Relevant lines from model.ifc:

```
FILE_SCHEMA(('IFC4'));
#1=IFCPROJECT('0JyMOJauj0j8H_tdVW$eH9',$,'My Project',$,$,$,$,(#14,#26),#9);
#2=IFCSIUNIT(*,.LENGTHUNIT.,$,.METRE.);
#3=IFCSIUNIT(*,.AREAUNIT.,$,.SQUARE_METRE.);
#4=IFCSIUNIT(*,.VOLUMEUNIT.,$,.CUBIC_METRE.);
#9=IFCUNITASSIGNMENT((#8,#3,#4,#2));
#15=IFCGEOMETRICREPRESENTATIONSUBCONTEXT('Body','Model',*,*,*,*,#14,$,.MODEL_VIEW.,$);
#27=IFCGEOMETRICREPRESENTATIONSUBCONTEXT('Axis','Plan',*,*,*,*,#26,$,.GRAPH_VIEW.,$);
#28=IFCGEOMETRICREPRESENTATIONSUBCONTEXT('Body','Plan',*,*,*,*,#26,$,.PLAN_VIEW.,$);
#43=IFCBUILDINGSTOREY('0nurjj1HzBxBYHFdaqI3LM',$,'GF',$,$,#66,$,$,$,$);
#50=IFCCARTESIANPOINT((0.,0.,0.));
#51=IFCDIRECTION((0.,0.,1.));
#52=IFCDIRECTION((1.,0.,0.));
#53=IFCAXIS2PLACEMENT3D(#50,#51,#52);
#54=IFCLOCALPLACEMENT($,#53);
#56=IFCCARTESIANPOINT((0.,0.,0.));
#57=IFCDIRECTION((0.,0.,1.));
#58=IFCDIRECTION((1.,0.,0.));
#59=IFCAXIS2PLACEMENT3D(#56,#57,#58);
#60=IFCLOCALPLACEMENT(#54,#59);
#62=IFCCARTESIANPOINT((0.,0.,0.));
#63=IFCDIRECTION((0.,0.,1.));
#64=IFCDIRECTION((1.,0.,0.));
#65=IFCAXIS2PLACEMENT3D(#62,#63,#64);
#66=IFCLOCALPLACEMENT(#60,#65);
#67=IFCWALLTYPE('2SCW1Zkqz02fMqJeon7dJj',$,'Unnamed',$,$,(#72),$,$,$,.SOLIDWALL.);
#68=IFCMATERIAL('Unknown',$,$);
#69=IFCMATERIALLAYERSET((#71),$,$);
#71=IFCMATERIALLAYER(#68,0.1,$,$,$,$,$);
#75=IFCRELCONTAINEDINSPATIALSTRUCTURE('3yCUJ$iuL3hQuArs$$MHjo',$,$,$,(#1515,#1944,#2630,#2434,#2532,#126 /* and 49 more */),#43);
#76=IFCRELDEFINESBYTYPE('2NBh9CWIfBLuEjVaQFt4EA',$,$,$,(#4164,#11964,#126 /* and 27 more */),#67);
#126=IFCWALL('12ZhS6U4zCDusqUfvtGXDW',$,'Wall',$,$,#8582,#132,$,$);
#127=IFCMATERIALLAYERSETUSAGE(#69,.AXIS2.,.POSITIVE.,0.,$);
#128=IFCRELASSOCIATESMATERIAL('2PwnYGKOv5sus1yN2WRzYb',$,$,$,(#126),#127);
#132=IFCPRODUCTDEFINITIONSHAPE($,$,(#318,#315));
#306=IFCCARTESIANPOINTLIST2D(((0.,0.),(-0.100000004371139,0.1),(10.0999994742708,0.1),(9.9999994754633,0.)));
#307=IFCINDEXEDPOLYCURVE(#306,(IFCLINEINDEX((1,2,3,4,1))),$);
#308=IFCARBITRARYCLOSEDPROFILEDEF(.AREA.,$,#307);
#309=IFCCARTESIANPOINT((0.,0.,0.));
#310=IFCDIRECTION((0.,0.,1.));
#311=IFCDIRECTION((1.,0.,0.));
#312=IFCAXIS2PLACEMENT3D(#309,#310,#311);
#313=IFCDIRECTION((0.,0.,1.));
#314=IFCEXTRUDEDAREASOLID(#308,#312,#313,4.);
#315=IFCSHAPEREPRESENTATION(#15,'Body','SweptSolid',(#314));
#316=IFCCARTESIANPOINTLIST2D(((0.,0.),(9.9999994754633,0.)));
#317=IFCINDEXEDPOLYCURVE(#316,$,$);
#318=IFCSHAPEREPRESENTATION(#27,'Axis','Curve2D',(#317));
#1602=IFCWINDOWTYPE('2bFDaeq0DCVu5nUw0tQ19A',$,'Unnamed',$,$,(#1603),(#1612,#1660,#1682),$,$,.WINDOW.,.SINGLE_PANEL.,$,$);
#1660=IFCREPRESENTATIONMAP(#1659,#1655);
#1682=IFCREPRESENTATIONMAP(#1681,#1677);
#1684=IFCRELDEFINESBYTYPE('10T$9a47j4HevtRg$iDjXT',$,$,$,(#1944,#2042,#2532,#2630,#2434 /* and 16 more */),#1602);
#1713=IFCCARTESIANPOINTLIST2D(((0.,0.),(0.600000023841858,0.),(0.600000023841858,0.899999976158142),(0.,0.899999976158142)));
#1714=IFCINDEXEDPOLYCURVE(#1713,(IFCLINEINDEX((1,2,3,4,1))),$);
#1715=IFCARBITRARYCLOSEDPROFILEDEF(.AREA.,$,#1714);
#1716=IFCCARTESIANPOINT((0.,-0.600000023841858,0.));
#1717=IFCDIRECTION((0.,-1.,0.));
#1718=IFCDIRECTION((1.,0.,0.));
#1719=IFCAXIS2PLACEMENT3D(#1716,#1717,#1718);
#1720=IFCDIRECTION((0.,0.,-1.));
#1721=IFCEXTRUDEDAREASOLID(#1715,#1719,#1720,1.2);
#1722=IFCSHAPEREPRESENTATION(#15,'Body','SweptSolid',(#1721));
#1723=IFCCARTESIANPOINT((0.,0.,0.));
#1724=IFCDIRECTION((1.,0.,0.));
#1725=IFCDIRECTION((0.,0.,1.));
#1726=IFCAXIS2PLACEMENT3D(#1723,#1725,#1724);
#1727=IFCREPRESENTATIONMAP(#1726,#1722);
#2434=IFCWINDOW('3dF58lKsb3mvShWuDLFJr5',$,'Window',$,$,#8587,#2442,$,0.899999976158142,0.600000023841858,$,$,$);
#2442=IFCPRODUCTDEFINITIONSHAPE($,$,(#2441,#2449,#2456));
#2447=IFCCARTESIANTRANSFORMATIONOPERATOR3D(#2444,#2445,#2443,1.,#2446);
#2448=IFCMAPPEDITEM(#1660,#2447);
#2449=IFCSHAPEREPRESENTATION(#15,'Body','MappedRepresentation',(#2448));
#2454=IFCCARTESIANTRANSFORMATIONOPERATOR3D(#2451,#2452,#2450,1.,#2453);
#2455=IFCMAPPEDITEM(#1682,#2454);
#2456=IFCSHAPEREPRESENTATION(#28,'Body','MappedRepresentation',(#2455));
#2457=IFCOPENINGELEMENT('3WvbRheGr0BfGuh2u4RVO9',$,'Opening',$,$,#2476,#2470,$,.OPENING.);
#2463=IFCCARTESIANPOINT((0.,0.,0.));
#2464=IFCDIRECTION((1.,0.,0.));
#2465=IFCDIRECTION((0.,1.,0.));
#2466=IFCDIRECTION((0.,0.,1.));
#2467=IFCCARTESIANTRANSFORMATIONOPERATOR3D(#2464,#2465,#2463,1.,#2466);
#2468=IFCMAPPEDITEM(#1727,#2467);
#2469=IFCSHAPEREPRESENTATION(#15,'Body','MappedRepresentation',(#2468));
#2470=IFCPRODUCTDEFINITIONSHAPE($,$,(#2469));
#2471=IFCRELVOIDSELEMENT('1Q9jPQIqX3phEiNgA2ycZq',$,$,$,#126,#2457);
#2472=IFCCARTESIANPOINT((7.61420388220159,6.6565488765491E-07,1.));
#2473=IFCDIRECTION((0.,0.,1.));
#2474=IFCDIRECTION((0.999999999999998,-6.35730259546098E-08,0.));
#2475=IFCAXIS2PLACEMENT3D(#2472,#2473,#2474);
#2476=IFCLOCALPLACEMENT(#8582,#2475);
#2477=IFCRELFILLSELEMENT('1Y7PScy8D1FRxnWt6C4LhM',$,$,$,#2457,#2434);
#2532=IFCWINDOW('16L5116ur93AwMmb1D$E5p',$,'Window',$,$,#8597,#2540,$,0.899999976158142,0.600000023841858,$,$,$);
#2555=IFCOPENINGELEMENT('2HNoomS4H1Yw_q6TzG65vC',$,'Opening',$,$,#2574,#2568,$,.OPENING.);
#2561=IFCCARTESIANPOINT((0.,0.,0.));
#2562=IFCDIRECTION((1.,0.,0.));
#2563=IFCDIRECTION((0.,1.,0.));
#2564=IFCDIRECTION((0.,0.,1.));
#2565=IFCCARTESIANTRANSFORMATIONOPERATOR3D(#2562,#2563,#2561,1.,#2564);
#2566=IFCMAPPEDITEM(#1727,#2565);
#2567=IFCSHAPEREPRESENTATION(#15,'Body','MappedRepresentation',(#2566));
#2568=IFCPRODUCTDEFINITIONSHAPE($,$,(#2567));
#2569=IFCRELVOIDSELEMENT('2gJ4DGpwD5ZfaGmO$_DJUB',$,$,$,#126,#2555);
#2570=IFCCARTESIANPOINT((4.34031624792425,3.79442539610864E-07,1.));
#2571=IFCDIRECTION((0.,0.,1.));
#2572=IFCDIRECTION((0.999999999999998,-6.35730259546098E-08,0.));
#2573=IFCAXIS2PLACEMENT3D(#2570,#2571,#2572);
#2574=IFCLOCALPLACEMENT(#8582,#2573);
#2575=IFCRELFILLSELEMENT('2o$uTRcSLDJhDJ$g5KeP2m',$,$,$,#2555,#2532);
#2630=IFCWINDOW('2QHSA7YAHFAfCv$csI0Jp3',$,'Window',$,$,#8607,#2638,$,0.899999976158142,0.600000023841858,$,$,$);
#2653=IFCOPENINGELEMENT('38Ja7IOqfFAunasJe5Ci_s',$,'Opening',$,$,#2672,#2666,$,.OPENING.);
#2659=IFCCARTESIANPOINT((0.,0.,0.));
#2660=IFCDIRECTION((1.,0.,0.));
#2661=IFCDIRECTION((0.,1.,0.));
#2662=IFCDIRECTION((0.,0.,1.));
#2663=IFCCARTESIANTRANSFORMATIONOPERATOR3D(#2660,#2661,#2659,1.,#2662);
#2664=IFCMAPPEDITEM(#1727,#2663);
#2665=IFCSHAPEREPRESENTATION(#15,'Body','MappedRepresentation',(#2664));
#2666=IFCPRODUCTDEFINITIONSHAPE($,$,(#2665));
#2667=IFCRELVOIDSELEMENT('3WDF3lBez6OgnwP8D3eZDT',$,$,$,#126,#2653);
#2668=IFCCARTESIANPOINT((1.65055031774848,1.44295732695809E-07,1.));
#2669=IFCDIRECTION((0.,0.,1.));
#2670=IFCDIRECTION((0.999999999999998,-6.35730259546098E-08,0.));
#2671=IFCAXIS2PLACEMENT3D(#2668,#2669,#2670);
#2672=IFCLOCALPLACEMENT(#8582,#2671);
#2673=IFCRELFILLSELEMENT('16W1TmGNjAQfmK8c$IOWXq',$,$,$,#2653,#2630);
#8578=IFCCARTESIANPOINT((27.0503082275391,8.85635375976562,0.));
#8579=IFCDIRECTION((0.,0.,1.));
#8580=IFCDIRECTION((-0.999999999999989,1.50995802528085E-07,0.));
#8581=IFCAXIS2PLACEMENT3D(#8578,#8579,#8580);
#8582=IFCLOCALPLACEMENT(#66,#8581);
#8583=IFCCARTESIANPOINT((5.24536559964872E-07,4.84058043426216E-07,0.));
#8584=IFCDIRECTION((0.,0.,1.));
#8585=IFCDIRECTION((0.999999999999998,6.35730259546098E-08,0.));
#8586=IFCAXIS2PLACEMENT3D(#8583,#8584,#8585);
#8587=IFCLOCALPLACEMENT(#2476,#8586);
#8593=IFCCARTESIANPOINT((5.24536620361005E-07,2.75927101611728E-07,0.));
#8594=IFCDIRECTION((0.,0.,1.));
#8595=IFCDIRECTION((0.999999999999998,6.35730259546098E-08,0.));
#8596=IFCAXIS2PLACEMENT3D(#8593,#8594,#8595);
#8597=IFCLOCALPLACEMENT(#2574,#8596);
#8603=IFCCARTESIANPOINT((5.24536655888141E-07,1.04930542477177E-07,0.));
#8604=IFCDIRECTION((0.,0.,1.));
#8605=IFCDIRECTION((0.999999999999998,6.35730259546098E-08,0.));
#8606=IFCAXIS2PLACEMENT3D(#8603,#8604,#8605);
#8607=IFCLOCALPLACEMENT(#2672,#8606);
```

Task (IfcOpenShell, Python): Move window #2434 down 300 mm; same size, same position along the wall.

```python
import numpy as np
import ifcopenshell
import ifcopenshell.api.geometry
import ifcopenshell.util.placement
import ifcopenshell.util.unit

model = ifcopenshell.open("model.ifc")
unit_scale = ifcopenshell.util.unit.calculate_unit_scale(model)

window = model.by_guid("3dF58lKsb3mvShWuDLFJr5")
opening = window.FillsVoids[0].RelatingOpeningElement
dz = -0.3

shift = np.array([0.0, 0.0, dz])
# The window is placed relative to its opening, so it follows when the opening moves.
matrix = ifcopenshell.util.placement.get_local_placement(opening.ObjectPlacement)
matrix[:3, 3] += shift
ifcopenshell.api.geometry.edit_object_placement(
    model, product=opening, matrix=matrix, is_si=False, should_transform_children=True
)

print(f"moved by {dz * unit_scale:+.3f} m")

model.write("model_updated.ifc")
```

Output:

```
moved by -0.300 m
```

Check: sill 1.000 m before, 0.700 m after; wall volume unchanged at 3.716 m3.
